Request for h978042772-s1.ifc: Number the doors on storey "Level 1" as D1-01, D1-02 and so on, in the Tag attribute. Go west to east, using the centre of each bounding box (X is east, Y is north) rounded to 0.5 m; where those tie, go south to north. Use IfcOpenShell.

First a look at what the model holds.

```python
import ifcopenshell
import ifcopenshell.util.element
import ifcopenshell.util.placement

model = ifcopenshell.open("h978042772-s1.ifc")
print(model.schema)
storey = next(s for s in model.by_type("IfcBuildingStorey") if s.Name == "Level 1")
doors = [e for e in ifcopenshell.util.element.get_decomposition(storey) if e.is_a("IfcDoor")]
for e in sorted(doors, key=lambda e: e.id()):
    origin = ifcopenshell.util.placement.get_local_placement(e.ObjectPlacement)[:3, 3]
    print(e.id(), e.Tag, e.Name, origin.round(2) + 0.0, sep=" | ")
```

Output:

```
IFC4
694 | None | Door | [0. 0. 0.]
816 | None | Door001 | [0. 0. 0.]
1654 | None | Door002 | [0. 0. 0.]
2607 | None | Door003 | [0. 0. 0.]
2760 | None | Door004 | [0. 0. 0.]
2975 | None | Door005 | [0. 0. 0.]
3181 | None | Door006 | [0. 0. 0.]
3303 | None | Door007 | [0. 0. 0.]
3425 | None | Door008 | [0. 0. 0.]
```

```python
import ifcopenshell
import ifcopenshell.geom
import ifcopenshell.util.element
import ifcopenshell.util.shape

model = ifcopenshell.open("h978042772-s1.ifc")
settings = ifcopenshell.geom.settings()
settings.set("use-world-coords", True)


def centre(element):
    shape = ifcopenshell.geom.create_shape(settings, element)
    return ifcopenshell.util.shape.get_bbox_centroid(shape.geometry)


storey = next(s for s in model.by_type("IfcBuildingStorey") if s.Name == "Level 1")
doors = [e for e in ifcopenshell.util.element.get_decomposition(storey) if e.is_a("IfcDoor")]

# Insertion points can sit at a corner or the storey origin, so sort by the geometry (in metres).
centres = {e: centre(e) for e in doors}
doors.sort(key=lambda e: (round(centres[e][0] / 0.5), centres[e][1]))

for i, e in enumerate(doors, start=1):
    number = f"D1-{i:02d}"
    e.Tag = number
    print(e.id(), number)

model.write("h978042772-s1_v2.ifc")
```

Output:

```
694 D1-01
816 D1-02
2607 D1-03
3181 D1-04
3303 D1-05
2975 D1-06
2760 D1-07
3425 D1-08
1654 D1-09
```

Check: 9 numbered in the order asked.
